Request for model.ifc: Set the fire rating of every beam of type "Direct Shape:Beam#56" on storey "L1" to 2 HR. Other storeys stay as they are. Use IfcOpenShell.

First a look at what the model holds.

```python
import ifcopenshell
import ifcopenshell.util.element

model = ifcopenshell.open("model.ifc")
print(model.schema)
storey = next(s for s in model.by_type("IfcBuildingStorey") if s.Name == "L1")
beams = [e for e in ifcopenshell.util.element.get_decomposition(storey) if e.is_a("IfcBeam")]
seen = {}
for e in beams:
    element_type = ifcopenshell.util.element.get_type(e)
    key = (element_type.Name if element_type != e and element_type else None, ifcopenshell.util.element.get_pset(e, "Pset_BeamCommon", "FireRating"))
    seen[key] = seen.get(key, 0) + 1
for (name, value), count in sorted(seen.items(), key=str):
    print(count, "x", name, "|", value)
```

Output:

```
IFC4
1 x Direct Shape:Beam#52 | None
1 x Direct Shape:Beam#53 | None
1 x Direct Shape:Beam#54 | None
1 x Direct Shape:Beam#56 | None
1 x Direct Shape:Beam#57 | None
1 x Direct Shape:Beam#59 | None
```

```python
import ifcopenshell
import ifcopenshell.api.pset
import ifcopenshell.util.element

model = ifcopenshell.open("model.ifc")

storey = next(s for s in model.by_type("IfcBuildingStorey") if s.Name == "L1")
beams = [e for e in ifcopenshell.util.element.get_decomposition(storey) if e.is_a("IfcBeam")]

count = 0
for e in beams:
    element_type = ifcopenshell.util.element.get_type(e)
    if element_type in (None, e) or element_type.Name != "Direct Shape:Beam#56":
        continue
    # add_pset returns the element's existing set when there is one.
    pset = ifcopenshell.api.pset.add_pset(model, product=e, name="Pset_BeamCommon")
    ifcopenshell.api.pset.edit_pset(model, pset=pset, properties={"FireRating": "2 HR"})
    count += 1

print(count, "beams updated")

model.write("model_rev.ifc")
```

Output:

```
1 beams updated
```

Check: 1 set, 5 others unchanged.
